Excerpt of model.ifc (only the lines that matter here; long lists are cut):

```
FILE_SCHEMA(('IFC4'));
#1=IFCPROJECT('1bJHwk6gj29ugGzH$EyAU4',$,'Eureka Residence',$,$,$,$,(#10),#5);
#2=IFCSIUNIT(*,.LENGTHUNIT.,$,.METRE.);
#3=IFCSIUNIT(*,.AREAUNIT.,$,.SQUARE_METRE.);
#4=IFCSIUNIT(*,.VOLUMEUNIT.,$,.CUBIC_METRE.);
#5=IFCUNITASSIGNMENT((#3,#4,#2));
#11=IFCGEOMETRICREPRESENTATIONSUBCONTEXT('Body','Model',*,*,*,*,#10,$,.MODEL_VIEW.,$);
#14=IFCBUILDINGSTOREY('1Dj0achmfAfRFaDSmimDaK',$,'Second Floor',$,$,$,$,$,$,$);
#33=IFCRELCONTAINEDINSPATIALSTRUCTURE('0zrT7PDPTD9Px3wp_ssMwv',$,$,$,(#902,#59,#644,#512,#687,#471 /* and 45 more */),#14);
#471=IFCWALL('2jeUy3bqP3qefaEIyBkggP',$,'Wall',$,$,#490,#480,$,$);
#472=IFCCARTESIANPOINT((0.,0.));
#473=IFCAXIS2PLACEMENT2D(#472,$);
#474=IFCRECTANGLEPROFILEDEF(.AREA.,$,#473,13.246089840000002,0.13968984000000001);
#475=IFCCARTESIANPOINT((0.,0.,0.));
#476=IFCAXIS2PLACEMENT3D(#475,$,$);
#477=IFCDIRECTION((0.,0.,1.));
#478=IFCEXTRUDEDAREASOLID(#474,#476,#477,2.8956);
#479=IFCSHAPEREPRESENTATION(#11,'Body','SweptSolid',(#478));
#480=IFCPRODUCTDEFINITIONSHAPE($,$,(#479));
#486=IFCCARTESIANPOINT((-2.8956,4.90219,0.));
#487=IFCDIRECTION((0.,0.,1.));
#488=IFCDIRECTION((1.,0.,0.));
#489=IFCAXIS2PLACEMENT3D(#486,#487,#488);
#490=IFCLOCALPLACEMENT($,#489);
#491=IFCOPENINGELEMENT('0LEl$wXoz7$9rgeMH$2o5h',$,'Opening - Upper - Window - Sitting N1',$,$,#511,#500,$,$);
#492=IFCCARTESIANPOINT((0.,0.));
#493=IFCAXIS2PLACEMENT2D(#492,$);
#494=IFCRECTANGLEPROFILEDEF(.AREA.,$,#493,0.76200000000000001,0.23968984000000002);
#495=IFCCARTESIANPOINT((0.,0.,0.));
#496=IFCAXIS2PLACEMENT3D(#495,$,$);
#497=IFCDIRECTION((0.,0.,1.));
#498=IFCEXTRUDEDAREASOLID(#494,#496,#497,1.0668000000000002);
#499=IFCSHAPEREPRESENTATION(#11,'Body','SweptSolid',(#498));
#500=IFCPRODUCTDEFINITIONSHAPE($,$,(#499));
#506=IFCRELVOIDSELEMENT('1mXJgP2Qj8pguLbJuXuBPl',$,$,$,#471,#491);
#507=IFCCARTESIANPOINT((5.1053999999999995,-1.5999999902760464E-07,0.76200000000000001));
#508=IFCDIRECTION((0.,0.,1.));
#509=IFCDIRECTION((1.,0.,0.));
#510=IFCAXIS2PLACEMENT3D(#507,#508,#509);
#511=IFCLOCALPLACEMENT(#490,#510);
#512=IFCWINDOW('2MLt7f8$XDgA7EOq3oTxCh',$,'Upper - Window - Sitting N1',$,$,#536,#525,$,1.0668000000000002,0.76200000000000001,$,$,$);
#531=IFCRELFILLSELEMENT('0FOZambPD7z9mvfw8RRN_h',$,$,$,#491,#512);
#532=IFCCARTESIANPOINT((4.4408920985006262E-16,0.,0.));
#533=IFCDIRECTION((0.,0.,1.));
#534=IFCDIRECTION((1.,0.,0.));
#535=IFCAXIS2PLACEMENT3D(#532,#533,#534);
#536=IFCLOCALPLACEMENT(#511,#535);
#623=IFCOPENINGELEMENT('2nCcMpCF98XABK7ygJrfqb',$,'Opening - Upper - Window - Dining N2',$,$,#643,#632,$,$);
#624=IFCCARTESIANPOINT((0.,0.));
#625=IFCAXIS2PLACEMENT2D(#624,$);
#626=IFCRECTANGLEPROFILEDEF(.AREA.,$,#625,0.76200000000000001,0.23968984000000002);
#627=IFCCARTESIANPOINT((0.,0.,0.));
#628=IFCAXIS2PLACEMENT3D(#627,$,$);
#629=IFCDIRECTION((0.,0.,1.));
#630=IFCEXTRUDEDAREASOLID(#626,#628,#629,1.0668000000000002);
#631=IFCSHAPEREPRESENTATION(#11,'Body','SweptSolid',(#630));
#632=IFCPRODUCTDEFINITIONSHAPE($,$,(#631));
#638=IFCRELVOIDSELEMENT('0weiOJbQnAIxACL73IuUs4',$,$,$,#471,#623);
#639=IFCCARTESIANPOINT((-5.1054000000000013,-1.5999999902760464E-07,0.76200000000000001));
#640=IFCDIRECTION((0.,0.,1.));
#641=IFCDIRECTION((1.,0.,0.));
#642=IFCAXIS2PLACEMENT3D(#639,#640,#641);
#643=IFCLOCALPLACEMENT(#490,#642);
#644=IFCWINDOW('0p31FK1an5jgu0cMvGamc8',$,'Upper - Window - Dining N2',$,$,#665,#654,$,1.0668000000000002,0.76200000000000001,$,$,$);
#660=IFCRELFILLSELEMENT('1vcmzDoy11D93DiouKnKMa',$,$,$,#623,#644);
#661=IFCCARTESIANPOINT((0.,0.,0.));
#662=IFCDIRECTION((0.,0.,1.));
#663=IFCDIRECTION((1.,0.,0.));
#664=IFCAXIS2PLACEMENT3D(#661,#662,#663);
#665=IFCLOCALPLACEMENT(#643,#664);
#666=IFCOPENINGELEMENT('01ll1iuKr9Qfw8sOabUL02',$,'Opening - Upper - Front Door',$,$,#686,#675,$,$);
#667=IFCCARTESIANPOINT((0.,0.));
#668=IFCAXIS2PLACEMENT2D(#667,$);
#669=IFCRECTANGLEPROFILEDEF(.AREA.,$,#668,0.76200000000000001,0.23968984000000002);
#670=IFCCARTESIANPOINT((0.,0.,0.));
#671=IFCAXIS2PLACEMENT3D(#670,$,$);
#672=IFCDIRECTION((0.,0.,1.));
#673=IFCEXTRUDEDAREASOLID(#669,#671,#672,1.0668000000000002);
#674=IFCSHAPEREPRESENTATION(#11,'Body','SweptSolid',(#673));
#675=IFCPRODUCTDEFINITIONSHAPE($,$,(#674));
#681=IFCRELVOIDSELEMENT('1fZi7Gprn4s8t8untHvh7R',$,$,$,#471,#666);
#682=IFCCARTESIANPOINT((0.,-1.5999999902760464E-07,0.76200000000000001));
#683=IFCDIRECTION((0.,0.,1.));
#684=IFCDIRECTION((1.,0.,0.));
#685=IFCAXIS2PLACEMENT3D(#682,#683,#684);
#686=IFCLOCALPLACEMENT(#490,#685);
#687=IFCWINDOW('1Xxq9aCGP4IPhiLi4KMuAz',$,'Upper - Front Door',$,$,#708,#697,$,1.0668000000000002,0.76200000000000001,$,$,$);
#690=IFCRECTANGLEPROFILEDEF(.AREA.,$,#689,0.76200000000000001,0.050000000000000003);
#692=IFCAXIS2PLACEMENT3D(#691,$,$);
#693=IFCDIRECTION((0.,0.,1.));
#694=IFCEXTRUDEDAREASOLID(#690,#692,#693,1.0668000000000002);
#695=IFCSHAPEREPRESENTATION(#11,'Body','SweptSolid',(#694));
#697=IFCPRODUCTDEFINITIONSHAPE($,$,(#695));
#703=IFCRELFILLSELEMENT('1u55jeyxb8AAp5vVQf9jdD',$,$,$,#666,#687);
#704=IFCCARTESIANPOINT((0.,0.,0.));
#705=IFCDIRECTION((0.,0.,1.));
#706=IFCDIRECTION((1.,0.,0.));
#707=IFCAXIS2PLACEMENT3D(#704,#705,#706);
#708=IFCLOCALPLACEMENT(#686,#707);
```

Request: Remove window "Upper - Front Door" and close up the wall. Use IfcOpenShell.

```python
import ifcopenshell
import ifcopenshell.api.feature
import ifcopenshell.api.root
import ifcopenshell.geom
import ifcopenshell.util.shape

model = ifcopenshell.open("model.ifc")
settings = ifcopenshell.geom.settings()


def volume(element):
    """Net volume in cubic metres, openings subtracted."""
    shape = ifcopenshell.geom.create_shape(settings, element)
    return ifcopenshell.util.shape.get_volume(shape.geometry)


window = model.by_guid("1Xxq9aCGP4IPhiLi4KMuAz")
opening = window.FillsVoids[0].RelatingOpeningElement
wall = opening.VoidsElements[0].RelatingBuildingElement
before = volume(wall)

ifcopenshell.api.root.remove_product(model, product=window)
ifcopenshell.api.feature.remove_feature(model, feature=opening)

after = volume(wall)

print(f"wall volume {before:.3f} -> {after:.3f} m3")

model.write("model_rev.ifc")
```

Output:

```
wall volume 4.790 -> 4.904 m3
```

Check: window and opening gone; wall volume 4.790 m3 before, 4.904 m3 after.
